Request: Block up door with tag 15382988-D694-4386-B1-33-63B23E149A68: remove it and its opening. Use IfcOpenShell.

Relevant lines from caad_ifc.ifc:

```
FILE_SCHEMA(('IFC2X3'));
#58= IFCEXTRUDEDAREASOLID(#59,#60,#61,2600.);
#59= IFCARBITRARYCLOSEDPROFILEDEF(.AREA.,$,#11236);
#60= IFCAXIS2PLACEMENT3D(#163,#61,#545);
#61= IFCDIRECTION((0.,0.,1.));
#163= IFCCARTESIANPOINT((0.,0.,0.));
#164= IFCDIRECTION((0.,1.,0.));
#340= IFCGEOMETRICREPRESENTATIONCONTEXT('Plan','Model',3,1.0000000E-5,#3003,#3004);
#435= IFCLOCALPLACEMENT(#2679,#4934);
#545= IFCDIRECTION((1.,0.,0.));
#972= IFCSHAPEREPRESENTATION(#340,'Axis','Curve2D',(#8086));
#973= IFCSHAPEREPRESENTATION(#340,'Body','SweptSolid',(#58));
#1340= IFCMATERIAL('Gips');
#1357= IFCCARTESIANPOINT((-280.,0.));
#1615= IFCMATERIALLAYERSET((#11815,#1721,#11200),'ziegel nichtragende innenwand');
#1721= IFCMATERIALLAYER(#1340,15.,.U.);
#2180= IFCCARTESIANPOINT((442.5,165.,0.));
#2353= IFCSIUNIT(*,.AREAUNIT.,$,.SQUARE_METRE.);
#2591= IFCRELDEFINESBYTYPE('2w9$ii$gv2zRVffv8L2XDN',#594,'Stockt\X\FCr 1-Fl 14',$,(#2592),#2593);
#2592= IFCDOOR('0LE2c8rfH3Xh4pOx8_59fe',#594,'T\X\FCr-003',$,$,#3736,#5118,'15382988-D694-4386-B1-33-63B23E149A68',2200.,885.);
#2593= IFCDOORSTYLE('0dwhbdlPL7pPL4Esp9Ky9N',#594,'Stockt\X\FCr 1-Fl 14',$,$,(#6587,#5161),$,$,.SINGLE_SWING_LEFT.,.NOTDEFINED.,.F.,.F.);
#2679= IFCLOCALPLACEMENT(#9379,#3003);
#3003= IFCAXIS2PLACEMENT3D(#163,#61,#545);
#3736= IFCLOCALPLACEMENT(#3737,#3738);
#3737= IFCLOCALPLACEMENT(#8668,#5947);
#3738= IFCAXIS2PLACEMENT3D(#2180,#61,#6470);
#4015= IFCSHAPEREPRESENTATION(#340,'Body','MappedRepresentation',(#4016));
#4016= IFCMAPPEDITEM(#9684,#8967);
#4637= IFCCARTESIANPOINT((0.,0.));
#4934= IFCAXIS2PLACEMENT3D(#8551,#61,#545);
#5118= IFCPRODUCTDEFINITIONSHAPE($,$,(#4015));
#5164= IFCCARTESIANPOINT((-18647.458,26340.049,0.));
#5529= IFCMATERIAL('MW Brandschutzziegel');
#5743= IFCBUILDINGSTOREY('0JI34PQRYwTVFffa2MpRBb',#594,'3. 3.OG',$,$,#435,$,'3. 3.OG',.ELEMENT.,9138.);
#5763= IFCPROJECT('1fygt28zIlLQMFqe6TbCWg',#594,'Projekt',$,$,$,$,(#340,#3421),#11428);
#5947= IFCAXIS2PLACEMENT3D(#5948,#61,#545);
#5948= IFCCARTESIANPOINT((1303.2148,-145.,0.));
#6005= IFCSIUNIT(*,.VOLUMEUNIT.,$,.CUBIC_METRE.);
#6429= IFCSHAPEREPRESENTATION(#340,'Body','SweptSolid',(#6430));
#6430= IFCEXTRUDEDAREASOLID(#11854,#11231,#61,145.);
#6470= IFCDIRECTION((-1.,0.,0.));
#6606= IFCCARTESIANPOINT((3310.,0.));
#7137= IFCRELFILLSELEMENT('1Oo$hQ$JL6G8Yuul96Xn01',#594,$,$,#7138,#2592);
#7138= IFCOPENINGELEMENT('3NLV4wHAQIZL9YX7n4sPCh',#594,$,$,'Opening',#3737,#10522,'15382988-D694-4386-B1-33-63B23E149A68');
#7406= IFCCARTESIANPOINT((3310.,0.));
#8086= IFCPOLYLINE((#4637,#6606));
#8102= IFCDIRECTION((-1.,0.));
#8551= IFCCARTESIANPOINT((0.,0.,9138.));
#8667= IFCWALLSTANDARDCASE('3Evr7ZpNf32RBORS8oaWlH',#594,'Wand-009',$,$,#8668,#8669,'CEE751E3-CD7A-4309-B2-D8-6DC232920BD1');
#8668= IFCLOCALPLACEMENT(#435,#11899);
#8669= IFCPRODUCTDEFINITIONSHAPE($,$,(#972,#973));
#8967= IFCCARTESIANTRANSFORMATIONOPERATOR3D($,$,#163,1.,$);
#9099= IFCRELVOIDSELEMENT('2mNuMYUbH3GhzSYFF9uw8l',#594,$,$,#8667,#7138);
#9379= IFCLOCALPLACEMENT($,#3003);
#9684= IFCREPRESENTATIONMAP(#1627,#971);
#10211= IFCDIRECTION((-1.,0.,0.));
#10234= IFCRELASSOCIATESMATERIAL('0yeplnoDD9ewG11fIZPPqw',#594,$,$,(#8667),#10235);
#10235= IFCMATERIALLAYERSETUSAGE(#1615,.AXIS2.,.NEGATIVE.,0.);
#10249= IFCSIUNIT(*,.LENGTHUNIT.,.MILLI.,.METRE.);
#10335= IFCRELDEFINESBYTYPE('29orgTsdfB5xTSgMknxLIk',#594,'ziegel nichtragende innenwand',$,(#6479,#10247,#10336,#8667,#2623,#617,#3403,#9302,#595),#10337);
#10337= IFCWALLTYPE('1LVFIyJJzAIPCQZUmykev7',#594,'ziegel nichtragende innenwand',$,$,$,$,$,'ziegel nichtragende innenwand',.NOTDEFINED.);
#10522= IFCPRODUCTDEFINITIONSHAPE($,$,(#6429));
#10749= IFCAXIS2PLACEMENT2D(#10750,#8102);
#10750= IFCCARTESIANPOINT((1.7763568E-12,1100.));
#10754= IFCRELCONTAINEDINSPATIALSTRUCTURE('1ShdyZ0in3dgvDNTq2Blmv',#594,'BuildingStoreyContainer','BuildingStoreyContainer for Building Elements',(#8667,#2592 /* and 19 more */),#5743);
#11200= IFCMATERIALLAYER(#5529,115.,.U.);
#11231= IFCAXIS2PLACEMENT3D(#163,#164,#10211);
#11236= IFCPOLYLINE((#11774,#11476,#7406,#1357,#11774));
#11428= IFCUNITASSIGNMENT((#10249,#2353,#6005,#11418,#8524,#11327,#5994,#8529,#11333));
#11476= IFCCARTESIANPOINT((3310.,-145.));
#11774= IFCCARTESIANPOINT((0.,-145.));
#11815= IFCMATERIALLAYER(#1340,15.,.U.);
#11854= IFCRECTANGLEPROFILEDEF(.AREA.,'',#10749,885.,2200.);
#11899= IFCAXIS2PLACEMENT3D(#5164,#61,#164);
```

```python
import ifcopenshell
import ifcopenshell.api.feature
import ifcopenshell.api.root
import ifcopenshell.geom
import ifcopenshell.util.shape

model = ifcopenshell.open("caad_ifc.ifc")
settings = ifcopenshell.geom.settings()


def volume(element):
    """Net volume in cubic metres, openings subtracted."""
    shape = ifcopenshell.geom.create_shape(settings, element)
    return ifcopenshell.util.shape.get_volume(shape.geometry)


door = model.by_guid("0LE2c8rfH3Xh4pOx8_59fe")
opening = door.FillsVoids[0].RelatingOpeningElement
wall = opening.VoidsElements[0].RelatingBuildingElement
before = volume(wall)

ifcopenshell.api.root.remove_product(model, product=door)
ifcopenshell.api.feature.remove_feature(model, feature=opening)

after = volume(wall)

print(f"wall volume {before:.3f} -> {after:.3f} m3")

model.write("caad_ifc-out.ifc")
```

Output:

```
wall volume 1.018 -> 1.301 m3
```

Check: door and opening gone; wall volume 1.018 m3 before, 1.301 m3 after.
